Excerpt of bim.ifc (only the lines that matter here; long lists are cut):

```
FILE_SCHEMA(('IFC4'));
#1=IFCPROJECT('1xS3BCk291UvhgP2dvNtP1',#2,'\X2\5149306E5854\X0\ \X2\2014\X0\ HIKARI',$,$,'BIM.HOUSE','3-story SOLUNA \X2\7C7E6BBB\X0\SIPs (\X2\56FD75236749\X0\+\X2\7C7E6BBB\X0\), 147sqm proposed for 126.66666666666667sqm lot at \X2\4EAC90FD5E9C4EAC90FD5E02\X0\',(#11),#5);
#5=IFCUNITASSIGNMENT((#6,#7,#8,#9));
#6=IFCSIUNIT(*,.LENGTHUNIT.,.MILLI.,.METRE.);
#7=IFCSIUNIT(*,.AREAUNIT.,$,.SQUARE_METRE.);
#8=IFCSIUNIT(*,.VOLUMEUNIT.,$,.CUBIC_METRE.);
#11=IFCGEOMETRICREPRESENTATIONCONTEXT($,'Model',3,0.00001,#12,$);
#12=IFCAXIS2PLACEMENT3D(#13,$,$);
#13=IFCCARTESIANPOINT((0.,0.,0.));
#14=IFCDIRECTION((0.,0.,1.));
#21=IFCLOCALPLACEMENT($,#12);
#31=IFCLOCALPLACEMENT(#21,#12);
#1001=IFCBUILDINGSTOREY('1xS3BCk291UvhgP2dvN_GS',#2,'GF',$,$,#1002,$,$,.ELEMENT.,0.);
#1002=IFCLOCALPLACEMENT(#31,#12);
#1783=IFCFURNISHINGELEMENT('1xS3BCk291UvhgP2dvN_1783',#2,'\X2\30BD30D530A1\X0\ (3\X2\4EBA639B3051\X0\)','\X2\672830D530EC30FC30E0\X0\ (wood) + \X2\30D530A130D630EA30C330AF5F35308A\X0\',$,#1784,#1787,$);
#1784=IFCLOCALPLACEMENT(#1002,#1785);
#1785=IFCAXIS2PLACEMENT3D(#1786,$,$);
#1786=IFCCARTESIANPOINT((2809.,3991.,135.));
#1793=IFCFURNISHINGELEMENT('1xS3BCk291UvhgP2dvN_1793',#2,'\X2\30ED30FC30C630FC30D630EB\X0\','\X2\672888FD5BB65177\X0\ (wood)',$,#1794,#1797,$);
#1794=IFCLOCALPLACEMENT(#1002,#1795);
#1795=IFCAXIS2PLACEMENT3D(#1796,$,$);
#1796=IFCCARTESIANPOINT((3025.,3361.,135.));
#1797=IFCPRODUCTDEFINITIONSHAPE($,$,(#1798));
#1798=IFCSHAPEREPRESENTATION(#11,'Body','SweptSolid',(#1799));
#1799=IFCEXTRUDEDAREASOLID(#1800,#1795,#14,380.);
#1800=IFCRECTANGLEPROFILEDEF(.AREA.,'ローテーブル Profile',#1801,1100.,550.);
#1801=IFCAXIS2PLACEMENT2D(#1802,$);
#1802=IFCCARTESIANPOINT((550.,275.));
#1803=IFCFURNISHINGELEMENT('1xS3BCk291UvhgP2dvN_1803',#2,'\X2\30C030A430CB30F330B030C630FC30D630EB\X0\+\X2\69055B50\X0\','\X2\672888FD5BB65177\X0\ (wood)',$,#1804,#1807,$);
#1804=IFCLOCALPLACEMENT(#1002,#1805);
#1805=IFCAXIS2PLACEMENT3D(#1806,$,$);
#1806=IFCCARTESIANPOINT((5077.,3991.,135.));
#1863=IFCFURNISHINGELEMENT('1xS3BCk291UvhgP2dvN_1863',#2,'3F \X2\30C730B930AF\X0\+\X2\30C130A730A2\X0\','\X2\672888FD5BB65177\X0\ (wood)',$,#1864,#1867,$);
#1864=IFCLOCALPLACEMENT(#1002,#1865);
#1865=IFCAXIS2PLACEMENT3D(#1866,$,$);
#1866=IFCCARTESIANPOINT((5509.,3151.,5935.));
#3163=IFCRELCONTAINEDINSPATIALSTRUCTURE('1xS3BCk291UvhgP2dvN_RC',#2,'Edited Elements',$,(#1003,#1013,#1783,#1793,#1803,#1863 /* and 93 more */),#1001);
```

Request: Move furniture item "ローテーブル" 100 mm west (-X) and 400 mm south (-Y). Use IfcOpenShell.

```python
import ifcopenshell
import ifcopenshell.api.geometry
import ifcopenshell.util.placement

model = ifcopenshell.open("bim.ifc")

item = model.by_guid("1xS3BCk291UvhgP2dvN_1793")
matrix = ifcopenshell.util.placement.get_local_placement(item.ObjectPlacement)
matrix[0, 3] -= 100.0
matrix[1, 3] -= 400.0
ifcopenshell.api.geometry.edit_object_placement(model, product=item, matrix=matrix, is_si=False)

print(ifcopenshell.util.placement.get_local_placement(item.ObjectPlacement).round(3) + 0.0)

model.write("bim_edited.ifc")
```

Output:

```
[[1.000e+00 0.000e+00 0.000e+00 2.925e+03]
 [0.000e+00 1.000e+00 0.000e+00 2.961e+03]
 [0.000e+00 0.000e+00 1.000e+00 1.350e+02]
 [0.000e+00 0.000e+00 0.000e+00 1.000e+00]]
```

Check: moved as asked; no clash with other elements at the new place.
